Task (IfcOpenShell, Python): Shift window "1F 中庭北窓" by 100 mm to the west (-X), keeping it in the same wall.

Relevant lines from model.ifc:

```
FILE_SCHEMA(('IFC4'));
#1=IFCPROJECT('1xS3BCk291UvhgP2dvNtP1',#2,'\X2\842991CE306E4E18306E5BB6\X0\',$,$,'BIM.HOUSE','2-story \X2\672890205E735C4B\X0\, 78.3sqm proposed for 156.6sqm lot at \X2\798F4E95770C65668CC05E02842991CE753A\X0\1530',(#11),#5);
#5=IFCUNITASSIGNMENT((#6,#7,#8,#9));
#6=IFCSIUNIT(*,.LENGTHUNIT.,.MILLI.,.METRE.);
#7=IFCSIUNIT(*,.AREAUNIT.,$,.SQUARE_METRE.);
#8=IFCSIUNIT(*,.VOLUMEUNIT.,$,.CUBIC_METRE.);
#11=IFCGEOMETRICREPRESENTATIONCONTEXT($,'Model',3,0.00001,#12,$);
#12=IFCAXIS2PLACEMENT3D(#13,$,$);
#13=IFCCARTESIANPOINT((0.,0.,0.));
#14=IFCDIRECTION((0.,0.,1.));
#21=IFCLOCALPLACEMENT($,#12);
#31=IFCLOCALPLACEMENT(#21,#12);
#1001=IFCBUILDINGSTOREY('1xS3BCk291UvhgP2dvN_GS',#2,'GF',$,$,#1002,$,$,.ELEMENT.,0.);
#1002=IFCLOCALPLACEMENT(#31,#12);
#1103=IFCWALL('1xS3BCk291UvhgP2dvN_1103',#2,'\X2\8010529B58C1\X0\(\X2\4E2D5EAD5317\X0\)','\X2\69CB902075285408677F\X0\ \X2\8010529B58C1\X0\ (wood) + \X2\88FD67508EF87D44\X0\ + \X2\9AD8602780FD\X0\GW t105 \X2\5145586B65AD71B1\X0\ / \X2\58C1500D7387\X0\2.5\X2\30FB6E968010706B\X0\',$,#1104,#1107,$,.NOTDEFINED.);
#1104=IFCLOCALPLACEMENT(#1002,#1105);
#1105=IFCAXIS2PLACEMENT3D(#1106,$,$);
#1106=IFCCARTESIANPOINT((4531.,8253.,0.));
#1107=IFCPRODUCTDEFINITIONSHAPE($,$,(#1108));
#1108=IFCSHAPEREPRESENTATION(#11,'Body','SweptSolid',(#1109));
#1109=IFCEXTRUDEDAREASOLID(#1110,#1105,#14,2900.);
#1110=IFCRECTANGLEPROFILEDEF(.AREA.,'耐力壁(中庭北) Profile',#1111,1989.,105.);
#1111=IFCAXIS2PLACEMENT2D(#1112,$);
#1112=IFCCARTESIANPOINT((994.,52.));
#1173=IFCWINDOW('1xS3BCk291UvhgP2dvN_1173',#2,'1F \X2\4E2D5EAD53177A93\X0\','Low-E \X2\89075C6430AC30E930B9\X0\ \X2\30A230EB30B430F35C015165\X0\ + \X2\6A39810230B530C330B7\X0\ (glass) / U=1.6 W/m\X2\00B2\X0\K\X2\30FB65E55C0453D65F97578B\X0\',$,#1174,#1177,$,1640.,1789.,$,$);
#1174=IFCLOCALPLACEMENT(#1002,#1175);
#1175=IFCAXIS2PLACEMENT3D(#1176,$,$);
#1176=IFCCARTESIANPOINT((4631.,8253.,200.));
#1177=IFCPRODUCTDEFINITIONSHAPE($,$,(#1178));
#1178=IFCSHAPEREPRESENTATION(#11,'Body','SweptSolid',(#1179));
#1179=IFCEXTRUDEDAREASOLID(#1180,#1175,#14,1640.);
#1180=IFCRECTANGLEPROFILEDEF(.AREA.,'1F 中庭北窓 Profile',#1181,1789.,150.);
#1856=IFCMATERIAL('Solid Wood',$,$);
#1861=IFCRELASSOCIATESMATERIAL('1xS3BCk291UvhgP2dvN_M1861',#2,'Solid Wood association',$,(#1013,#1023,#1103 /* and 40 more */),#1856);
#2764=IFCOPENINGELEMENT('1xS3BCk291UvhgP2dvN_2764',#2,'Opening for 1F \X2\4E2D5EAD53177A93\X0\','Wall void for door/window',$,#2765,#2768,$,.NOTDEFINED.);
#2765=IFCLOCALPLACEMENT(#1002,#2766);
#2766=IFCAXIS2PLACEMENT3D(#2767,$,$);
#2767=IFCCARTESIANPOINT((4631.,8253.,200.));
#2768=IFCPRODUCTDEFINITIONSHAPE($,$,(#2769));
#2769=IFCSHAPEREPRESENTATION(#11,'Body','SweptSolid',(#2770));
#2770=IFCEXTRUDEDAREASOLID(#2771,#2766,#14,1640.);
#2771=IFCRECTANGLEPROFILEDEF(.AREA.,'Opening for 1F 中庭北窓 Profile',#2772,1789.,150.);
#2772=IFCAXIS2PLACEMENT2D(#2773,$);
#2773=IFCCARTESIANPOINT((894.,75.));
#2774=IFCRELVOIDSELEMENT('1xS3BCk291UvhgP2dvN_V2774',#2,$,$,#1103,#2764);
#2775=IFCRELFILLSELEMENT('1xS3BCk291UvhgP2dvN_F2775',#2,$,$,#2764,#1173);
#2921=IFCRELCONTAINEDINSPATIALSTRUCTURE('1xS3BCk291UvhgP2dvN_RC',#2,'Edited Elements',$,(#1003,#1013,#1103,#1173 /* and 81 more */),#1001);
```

```python
import ifcopenshell
import ifcopenshell.api.geometry
import ifcopenshell.util.placement

model = ifcopenshell.open("model.ifc")

window = model.by_guid("1xS3BCk291UvhgP2dvN_1173")
opening = window.FillsVoids[0].RelatingOpeningElement
wall = opening.VoidsElements[0].RelatingBuildingElement

wall_matrix = ifcopenshell.util.placement.get_local_placement(wall.ObjectPlacement)
shift = wall_matrix[:3, 0] * -100.0
before = ifcopenshell.util.placement.get_local_placement(window.ObjectPlacement)[:3, 3].copy()

# The window is not placed relative to its opening, so move both.
for product in (opening, window):
    matrix = ifcopenshell.util.placement.get_local_placement(product.ObjectPlacement)
    matrix[:3, 3] += shift
    ifcopenshell.api.geometry.edit_object_placement(model, product=product, matrix=matrix, is_si=False)

after = ifcopenshell.util.placement.get_local_placement(window.ObjectPlacement)[:3, 3]
print("window moved by", (after - before).round(3) + 0.0)

model.write("model_updated.ifc")
```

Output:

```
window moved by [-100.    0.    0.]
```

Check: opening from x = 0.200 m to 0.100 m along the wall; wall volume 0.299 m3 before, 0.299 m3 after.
